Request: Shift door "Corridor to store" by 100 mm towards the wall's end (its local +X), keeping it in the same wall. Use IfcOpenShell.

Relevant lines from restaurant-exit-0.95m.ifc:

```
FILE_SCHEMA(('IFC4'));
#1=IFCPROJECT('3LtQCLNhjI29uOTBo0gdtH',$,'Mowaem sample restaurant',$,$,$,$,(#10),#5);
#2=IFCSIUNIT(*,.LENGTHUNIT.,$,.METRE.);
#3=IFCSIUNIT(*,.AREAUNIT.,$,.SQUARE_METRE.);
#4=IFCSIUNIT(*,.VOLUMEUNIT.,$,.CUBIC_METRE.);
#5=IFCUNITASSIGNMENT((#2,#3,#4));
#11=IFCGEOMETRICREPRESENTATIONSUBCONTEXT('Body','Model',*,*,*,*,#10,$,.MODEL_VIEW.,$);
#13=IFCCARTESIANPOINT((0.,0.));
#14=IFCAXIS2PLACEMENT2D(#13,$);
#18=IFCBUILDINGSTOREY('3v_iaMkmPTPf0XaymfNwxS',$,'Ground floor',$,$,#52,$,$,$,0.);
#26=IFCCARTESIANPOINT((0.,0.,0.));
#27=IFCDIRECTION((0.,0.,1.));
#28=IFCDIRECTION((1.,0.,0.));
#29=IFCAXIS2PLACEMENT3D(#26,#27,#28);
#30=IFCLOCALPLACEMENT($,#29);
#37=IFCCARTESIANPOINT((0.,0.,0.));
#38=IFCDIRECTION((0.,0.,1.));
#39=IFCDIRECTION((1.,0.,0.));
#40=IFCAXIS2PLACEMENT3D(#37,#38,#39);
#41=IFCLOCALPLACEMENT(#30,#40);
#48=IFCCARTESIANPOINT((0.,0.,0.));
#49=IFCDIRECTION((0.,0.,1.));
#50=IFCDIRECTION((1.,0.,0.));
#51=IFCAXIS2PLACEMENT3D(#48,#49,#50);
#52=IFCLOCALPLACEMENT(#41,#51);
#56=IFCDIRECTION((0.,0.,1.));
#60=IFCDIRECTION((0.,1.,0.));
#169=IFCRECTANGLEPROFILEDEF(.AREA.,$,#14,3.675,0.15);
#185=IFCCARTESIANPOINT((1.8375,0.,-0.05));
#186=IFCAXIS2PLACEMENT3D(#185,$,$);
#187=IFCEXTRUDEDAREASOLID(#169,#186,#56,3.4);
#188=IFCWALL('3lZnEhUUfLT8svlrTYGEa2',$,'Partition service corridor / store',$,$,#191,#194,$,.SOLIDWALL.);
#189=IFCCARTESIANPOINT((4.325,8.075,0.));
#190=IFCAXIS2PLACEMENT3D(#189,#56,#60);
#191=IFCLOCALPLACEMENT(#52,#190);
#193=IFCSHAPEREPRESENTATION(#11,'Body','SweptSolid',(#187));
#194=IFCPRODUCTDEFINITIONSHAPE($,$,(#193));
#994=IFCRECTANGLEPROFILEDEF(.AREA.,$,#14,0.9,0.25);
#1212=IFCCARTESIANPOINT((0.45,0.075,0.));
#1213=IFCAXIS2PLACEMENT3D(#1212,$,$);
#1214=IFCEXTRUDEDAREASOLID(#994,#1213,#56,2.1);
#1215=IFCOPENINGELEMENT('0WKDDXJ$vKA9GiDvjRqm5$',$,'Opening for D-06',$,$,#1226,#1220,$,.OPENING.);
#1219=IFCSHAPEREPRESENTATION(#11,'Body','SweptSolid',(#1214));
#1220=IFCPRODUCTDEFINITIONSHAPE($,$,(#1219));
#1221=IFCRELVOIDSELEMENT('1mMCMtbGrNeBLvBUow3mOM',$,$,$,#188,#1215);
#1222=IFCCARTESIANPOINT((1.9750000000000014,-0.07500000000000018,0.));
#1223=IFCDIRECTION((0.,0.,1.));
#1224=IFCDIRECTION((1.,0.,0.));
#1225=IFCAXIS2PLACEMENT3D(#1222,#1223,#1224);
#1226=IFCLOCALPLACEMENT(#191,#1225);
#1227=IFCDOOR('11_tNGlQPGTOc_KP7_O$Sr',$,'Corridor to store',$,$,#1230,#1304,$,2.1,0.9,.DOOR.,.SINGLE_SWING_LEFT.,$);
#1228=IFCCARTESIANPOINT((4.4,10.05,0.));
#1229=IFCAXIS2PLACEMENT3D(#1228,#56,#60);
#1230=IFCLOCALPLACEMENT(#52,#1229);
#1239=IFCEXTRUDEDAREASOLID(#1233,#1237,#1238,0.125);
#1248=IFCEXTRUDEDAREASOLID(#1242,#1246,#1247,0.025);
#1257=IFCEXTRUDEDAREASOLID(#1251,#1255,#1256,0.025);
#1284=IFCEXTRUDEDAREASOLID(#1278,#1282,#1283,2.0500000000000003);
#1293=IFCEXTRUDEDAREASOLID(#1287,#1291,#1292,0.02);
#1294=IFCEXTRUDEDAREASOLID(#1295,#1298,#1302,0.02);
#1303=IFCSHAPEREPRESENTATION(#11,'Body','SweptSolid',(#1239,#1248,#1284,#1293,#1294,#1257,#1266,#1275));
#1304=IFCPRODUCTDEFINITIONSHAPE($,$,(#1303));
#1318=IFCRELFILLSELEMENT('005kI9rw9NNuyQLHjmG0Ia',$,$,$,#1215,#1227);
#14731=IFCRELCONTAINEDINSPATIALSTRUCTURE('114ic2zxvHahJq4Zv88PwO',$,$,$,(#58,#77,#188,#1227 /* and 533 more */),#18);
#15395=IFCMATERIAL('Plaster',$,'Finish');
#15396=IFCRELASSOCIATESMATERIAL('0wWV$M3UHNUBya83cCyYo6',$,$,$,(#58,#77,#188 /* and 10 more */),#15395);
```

```python
import ifcopenshell
import ifcopenshell.api.geometry
import ifcopenshell.util.placement
import ifcopenshell.util.unit

model = ifcopenshell.open("restaurant-exit-0.95m.ifc")
unit_scale = ifcopenshell.util.unit.calculate_unit_scale(model)

door = model.by_id(1227)
opening = door.FillsVoids[0].RelatingOpeningElement
wall = opening.VoidsElements[0].RelatingBuildingElement

wall_matrix = ifcopenshell.util.placement.get_local_placement(wall.ObjectPlacement)
shift = wall_matrix[:3, 0] * 0.1 / unit_scale
before = ifcopenshell.util.placement.get_local_placement(door.ObjectPlacement)[:3, 3].copy()

# The door is not placed relative to its opening, so move both.
for product in (opening, door):
    matrix = ifcopenshell.util.placement.get_local_placement(product.ObjectPlacement)
    matrix[:3, 3] += shift
    ifcopenshell.api.geometry.edit_object_placement(model, product=product, matrix=matrix, is_si=False)

after = ifcopenshell.util.placement.get_local_placement(door.ObjectPlacement)[:3, 3]
print("door moved by", (after - before).round(3) + 0.0)

model.write("restaurant-exit-0.95m_edited.ifc")
```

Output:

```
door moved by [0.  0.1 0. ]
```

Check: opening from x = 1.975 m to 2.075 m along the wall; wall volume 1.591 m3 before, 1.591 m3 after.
